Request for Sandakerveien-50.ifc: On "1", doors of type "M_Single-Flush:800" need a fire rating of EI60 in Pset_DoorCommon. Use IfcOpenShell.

First a look at what the model holds.

```python
import ifcopenshell
import ifcopenshell.util.element

model = ifcopenshell.open("Sandakerveien-50.ifc")
print(model.schema)
storey = next(s for s in model.by_type("IfcBuildingStorey") if s.Name == "1")
doors = [e for e in ifcopenshell.util.element.get_decomposition(storey) if e.is_a("IfcDoor")]
seen = {}
for e in doors:
    element_type = ifcopenshell.util.element.get_type(e)
    key = (element_type.Name if element_type != e and element_type else None, ifcopenshell.util.element.get_pset(e, "Pset_DoorCommon", "FireRating"))
    seen[key] = seen.get(key, 0) + 1
for (name, value), count in sorted(seen.items(), key=str):
    print(count, "x", name, "|", value)
```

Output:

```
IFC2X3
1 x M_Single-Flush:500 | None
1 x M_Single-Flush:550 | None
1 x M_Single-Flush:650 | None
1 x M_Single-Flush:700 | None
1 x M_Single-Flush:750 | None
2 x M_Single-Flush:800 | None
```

```python
import ifcopenshell
import ifcopenshell.api.pset
import ifcopenshell.util.element

model = ifcopenshell.open("Sandakerveien-50.ifc")

storey = next(s for s in model.by_type("IfcBuildingStorey") if s.Name == "1")
doors = [e for e in ifcopenshell.util.element.get_decomposition(storey) if e.is_a("IfcDoor")]

count = 0
for e in doors:
    element_type = ifcopenshell.util.element.get_type(e)
    if element_type in (None, e) or element_type.Name != "M_Single-Flush:800":
        continue
    # add_pset returns the element's existing set when there is one.
    pset = ifcopenshell.api.pset.add_pset(model, product=e, name="Pset_DoorCommon")
    ifcopenshell.api.pset.edit_pset(model, pset=pset, properties={"FireRating": "EI60"})
    count += 1

print(count, "doors updated")

model.write("Sandakerveien-50_rev.ifc")
```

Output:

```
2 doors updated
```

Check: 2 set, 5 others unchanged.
